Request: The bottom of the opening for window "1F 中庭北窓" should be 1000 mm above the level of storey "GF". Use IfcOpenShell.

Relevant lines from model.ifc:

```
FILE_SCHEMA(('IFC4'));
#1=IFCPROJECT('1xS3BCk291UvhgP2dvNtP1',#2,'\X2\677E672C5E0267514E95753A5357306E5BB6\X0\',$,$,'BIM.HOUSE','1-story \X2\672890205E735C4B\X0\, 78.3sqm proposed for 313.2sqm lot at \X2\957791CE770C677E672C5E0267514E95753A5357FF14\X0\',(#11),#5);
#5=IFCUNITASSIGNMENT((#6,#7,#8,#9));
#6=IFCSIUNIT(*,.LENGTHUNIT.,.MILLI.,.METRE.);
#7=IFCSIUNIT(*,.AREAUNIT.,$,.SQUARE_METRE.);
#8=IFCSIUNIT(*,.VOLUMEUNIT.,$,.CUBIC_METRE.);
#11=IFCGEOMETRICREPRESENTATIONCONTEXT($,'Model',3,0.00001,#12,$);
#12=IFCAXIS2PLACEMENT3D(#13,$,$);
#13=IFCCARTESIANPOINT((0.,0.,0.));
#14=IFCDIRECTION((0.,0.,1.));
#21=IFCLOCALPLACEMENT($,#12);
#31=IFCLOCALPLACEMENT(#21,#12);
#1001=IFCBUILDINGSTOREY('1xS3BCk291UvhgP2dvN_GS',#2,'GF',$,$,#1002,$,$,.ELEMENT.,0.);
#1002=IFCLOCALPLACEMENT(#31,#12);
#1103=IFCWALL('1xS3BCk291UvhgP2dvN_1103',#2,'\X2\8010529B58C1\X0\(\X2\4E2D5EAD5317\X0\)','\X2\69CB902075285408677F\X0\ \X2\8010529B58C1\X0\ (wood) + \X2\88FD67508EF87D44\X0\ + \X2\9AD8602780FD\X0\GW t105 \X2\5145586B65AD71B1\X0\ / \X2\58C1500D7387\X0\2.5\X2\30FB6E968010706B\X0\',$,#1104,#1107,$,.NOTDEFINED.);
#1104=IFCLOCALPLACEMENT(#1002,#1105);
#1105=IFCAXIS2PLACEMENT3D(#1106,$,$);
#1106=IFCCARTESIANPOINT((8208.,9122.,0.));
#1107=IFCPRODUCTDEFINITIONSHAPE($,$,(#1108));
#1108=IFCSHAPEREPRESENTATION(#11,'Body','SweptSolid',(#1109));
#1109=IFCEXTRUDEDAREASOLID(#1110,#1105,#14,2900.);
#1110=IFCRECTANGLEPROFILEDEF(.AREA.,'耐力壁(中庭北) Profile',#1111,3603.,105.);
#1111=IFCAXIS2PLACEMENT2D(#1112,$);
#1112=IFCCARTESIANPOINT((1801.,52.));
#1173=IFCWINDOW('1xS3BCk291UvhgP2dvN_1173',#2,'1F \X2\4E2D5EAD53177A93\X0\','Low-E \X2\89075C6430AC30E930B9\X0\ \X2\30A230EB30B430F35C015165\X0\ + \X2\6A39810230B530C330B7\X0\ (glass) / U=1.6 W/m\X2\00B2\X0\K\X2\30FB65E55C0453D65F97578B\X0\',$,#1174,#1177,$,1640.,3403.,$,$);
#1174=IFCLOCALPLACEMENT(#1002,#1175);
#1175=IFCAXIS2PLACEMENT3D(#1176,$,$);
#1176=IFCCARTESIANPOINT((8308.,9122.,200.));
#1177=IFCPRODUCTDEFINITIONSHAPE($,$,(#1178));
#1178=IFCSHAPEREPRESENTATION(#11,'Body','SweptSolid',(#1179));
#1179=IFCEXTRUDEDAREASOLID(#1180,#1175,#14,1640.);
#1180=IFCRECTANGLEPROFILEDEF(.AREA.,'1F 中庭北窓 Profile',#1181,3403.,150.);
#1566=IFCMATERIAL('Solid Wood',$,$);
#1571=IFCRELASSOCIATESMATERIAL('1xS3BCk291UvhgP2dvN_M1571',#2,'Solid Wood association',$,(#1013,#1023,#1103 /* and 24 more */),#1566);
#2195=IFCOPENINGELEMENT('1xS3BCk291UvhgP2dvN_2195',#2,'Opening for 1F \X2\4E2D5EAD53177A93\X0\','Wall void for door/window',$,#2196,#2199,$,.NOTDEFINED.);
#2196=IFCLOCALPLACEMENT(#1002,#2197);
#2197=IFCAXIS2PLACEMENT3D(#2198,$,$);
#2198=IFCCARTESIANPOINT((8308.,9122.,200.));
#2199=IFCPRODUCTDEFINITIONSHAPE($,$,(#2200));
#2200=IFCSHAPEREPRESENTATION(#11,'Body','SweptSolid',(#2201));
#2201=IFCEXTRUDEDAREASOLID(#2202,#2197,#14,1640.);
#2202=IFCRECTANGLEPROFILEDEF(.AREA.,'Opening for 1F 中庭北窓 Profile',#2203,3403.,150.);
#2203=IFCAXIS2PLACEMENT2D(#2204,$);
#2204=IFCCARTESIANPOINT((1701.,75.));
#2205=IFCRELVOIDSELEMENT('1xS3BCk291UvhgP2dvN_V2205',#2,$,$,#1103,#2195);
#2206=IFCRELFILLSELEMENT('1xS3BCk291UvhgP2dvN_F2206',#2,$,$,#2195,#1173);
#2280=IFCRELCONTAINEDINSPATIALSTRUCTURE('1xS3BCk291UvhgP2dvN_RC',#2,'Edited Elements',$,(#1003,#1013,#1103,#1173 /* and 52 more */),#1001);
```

```python
import numpy as np
import ifcopenshell
import ifcopenshell.api.geometry
import ifcopenshell.geom
import ifcopenshell.util.element
import ifcopenshell.util.placement
import ifcopenshell.util.shape
import ifcopenshell.util.unit

model = ifcopenshell.open("model.ifc")
unit_scale = ifcopenshell.util.unit.calculate_unit_scale(model)

window = model.by_id(1173)
opening = window.FillsVoids[0].RelatingOpeningElement
storey = ifcopenshell.util.element.get_container(window, ifc_class="IfcBuildingStorey")
level = ifcopenshell.util.placement.get_local_placement(storey.ObjectPlacement)[2, 3]

# The opening's origin need not be at the sill, so measure its lowest point.
shape = ifcopenshell.geom.create_shape(ifcopenshell.geom.settings(), opening)
bottom = ifcopenshell.util.shape.get_shape_bottom_elevation(shape, shape.geometry) / unit_scale
dz = level + 1000.0 - bottom

shift = np.array([0.0, 0.0, dz])
# The window is not placed relative to its opening, so move both.
for product in (opening, window):
    matrix = ifcopenshell.util.placement.get_local_placement(product.ObjectPlacement)
    matrix[:3, 3] += shift
    ifcopenshell.api.geometry.edit_object_placement(model, product=product, matrix=matrix, is_si=False)

print(f"moved by {dz * unit_scale:+.3f} m")

model.write("model_edited.ifc")
```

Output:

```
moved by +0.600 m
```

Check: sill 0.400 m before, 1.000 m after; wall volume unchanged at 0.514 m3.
